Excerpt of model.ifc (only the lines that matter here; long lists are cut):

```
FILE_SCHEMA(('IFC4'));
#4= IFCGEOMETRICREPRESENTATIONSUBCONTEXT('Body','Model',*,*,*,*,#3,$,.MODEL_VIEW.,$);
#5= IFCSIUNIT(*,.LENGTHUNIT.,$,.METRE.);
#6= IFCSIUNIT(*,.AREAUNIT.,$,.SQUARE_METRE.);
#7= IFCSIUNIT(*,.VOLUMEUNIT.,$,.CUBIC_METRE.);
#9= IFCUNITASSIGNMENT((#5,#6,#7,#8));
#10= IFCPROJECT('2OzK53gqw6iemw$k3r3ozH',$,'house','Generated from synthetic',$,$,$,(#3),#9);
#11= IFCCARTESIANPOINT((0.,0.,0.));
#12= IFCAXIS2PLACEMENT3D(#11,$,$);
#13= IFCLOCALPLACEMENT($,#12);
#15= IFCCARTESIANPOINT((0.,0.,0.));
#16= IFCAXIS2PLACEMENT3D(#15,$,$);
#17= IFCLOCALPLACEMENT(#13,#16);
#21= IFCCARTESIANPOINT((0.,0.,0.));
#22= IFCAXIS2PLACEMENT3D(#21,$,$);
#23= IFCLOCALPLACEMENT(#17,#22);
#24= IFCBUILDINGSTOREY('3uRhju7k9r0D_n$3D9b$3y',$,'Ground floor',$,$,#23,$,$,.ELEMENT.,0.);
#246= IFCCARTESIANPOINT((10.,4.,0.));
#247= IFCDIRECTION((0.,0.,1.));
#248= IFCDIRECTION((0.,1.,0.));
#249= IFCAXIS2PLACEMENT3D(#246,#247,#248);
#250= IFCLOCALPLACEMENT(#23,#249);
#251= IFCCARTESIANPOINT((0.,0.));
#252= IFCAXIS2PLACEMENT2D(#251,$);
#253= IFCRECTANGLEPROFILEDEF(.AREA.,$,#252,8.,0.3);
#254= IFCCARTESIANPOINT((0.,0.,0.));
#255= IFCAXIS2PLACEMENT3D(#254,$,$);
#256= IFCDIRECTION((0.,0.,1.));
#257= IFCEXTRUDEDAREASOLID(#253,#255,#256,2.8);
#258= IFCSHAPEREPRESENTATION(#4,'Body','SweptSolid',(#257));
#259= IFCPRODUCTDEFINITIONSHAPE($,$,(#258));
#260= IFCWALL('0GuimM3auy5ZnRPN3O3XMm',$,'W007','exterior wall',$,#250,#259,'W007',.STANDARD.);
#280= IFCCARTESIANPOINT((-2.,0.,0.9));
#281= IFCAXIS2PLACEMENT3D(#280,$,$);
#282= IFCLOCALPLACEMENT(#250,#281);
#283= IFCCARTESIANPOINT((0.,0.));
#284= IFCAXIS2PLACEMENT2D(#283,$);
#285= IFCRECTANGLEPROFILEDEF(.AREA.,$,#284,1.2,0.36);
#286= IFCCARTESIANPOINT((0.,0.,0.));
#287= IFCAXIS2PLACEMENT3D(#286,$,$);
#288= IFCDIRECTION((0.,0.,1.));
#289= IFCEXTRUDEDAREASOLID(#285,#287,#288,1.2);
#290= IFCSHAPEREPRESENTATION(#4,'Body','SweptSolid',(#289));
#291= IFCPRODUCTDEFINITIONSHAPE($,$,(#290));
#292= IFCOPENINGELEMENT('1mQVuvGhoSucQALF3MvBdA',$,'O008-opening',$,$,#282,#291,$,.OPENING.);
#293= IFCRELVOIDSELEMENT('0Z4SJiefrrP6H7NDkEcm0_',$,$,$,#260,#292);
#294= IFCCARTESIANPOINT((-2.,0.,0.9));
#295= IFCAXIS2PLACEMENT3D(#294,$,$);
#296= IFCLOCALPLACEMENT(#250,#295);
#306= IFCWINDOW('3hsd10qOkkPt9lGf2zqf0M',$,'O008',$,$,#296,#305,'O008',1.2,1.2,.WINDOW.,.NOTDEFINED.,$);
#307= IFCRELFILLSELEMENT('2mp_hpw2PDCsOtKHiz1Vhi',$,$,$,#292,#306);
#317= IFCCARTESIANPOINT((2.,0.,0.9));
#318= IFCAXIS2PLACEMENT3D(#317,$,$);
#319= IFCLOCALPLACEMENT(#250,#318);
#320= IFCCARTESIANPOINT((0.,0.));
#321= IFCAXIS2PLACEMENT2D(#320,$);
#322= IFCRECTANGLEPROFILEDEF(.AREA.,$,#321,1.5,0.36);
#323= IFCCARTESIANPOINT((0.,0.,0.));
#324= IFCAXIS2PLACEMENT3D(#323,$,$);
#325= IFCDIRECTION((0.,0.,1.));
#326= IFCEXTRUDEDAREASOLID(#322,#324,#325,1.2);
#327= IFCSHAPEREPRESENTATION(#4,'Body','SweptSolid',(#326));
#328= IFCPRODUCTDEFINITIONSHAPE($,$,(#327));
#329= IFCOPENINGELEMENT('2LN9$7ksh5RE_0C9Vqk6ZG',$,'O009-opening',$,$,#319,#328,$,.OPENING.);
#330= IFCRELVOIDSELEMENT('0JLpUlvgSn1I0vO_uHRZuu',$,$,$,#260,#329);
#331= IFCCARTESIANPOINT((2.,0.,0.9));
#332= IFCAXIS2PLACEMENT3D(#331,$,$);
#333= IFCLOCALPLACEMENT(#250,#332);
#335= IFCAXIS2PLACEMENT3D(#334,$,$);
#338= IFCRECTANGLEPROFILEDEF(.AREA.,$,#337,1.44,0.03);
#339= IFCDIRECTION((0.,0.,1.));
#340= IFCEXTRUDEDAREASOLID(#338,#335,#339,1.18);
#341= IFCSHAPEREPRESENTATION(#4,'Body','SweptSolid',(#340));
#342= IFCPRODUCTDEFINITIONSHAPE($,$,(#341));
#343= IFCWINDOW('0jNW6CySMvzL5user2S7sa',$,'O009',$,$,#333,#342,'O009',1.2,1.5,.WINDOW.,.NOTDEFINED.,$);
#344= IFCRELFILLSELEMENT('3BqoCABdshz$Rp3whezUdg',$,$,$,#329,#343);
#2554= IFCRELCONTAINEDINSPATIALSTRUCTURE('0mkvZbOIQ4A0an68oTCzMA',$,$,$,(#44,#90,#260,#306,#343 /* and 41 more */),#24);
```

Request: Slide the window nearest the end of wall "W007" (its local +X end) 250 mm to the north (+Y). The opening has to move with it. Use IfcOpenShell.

```python
import ifcopenshell
import ifcopenshell.api.geometry
import ifcopenshell.util.placement

model = ifcopenshell.open("model.ifc")

window = model.by_guid("0jNW6CySMvzL5user2S7sa")
opening = window.FillsVoids[0].RelatingOpeningElement
wall = opening.VoidsElements[0].RelatingBuildingElement

wall_matrix = ifcopenshell.util.placement.get_local_placement(wall.ObjectPlacement)
shift = wall_matrix[:3, 0] * 0.25
before = ifcopenshell.util.placement.get_local_placement(window.ObjectPlacement)[:3, 3].copy()

# The window is not placed relative to its opening, so move both.
for product in (opening, window):
    matrix = ifcopenshell.util.placement.get_local_placement(product.ObjectPlacement)
    matrix[:3, 3] += shift
    ifcopenshell.api.geometry.edit_object_placement(model, product=product, matrix=matrix, is_si=False)

after = ifcopenshell.util.placement.get_local_placement(window.ObjectPlacement)[:3, 3]
print("window moved by", (after - before).round(3) + 0.0)

model.write("model_v2.ifc")
```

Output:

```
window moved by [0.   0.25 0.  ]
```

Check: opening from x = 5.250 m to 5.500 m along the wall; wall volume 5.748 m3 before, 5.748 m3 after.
